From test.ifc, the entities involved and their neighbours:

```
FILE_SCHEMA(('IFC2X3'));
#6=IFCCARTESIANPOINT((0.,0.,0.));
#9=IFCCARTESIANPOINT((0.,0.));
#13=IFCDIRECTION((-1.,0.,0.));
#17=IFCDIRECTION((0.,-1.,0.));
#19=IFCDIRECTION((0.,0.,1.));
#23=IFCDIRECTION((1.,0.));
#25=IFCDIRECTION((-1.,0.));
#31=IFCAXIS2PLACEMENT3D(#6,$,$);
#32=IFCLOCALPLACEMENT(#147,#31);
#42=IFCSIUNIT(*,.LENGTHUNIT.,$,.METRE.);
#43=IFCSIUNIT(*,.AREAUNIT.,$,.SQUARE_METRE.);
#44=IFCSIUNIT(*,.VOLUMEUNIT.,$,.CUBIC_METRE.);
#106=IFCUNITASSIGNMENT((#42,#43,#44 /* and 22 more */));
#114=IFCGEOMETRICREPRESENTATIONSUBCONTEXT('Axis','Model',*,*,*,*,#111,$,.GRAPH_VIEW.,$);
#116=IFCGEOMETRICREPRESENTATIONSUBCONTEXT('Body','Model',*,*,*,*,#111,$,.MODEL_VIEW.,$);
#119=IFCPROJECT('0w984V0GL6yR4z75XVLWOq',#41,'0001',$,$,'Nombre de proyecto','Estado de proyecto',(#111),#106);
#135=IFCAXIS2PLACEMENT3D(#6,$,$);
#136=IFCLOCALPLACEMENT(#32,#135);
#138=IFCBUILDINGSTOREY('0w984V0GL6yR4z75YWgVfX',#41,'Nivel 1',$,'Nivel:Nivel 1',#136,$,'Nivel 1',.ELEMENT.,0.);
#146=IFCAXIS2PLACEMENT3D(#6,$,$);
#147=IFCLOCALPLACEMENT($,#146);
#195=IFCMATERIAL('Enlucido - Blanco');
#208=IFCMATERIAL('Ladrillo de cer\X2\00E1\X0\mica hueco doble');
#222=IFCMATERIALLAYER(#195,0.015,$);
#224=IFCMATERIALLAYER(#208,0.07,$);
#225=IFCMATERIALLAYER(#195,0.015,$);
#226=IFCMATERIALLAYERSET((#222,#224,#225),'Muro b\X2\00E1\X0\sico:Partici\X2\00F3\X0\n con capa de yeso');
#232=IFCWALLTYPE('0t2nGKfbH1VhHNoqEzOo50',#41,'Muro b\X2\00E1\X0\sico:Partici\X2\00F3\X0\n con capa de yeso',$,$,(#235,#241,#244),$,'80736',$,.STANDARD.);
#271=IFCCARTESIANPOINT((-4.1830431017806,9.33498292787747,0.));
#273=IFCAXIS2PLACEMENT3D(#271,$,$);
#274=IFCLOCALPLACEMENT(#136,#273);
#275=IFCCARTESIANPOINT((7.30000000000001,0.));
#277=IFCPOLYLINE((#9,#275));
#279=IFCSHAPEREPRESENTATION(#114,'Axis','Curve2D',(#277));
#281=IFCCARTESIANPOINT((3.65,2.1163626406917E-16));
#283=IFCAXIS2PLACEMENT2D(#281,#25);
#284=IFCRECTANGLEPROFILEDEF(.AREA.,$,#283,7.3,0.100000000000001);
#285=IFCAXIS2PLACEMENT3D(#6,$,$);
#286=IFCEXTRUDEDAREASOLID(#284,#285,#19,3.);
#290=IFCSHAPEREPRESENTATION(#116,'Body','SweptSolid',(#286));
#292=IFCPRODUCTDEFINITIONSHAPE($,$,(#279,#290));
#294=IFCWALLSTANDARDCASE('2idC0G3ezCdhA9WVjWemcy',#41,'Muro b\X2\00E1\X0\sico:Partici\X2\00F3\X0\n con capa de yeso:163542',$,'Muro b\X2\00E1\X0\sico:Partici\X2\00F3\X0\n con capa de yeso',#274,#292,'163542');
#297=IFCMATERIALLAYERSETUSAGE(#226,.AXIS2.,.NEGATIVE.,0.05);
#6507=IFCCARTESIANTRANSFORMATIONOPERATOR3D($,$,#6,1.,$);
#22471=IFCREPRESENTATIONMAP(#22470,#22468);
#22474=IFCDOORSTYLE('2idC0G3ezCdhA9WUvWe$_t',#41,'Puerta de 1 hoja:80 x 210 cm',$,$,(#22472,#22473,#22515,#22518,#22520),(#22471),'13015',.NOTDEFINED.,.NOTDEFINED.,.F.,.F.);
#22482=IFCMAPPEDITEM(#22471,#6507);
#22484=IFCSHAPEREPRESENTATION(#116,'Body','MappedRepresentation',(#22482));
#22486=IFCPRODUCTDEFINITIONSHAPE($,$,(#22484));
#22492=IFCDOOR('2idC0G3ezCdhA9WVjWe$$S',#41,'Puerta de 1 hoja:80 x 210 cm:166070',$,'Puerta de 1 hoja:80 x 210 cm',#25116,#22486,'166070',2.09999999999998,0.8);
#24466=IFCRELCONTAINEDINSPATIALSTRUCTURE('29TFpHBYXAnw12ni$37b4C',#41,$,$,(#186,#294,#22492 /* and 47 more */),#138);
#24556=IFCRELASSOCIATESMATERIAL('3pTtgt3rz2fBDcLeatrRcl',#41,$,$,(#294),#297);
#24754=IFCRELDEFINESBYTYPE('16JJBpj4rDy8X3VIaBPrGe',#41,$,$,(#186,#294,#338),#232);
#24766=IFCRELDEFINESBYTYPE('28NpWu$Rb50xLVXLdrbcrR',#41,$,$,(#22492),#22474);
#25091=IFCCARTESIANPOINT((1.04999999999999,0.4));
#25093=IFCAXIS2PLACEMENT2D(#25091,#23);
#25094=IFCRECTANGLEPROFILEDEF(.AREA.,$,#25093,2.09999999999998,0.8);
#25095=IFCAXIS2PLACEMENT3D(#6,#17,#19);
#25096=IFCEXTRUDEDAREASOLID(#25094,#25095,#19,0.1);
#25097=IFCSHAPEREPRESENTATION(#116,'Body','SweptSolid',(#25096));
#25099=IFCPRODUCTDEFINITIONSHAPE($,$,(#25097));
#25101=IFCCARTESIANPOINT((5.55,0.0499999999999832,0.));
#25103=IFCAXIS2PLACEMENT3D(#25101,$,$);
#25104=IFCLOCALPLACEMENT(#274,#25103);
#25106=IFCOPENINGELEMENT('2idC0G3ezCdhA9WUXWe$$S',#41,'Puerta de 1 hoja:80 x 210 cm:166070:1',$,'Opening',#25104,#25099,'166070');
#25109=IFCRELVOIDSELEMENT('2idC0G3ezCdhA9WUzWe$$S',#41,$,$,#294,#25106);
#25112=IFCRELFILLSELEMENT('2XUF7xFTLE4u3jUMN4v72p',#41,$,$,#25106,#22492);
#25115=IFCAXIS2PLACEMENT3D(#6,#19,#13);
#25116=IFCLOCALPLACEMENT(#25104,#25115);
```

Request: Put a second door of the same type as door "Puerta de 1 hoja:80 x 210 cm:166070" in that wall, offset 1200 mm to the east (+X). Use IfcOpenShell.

```python
import ifcopenshell
import ifcopenshell.api.feature
import ifcopenshell.api.geometry
import ifcopenshell.api.root
import ifcopenshell.geom
import ifcopenshell.util.element
import ifcopenshell.util.placement
import ifcopenshell.util.shape
import ifcopenshell.util.unit

model = ifcopenshell.open("test.ifc")
unit_scale = ifcopenshell.util.unit.calculate_unit_scale(model)
settings = ifcopenshell.geom.settings()


def volume(element):
    """Net volume in cubic metres, openings subtracted."""
    shape = ifcopenshell.geom.create_shape(settings, element)
    return ifcopenshell.util.shape.get_volume(shape.geometry)


def reuse_history(source, copy):
    """copy_class also copies each property set's owner history, people and application; keep the originals."""
    for rel in copy.IsDefinedBy:
        if rel.is_a("IfcRelDefinesByProperties") and (history := rel.RelatingPropertyDefinition.OwnerHistory):
            rel.RelatingPropertyDefinition.OwnerHistory = source.OwnerHistory
            ifcopenshell.util.element.remove_deep2(model, history)


door = model.by_guid("2idC0G3ezCdhA9WVjWe$$S")
opening = door.FillsVoids[0].RelatingOpeningElement
wall = opening.VoidsElements[0].RelatingBuildingElement
before = volume(wall)
shift = ifcopenshell.util.placement.get_local_placement(wall.ObjectPlacement)[:3, 0] * 1.2 / unit_scale

# copy_class copies the void relationship, type, container and properties, but no geometry.
new_opening = ifcopenshell.api.root.copy_class(model, product=opening)
new_opening.Representation = ifcopenshell.util.element.copy_deep(
    model, opening.Representation, exclude=["IfcGeometricRepresentationContext", "IfcRepresentationMap"]
)
new_opening.Name = "Puerta de 1 hoja:80 x 210 cm"
new_opening.Tag = None
new_door = ifcopenshell.api.root.copy_class(model, product=door)
new_door.Representation = ifcopenshell.util.element.copy_deep(
    model, door.Representation, exclude=["IfcGeometricRepresentationContext", "IfcRepresentationMap"]
)
new_door.Name = "Puerta de 1 hoja:80 x 210 cm"
new_door.Tag = None
reuse_history(door, new_door)
fills = ifcopenshell.api.feature.add_filling(model, opening=new_opening, element=new_door)
fills.OwnerHistory = new_door.OwnerHistory  # required in IFC2X3

for old, new in ((opening, new_opening), (door, new_door)):
    matrix = ifcopenshell.util.placement.get_local_placement(old.ObjectPlacement)
    matrix[:3, 3] += shift
    ifcopenshell.api.geometry.edit_object_placement(model, product=new, matrix=matrix, is_si=False)

after = volume(wall)

print(f"wall volume {before:.3f} -> {after:.3f} m3")

model.write("test_updated.ifc")
```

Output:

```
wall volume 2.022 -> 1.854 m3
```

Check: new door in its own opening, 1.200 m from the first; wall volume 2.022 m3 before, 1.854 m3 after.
